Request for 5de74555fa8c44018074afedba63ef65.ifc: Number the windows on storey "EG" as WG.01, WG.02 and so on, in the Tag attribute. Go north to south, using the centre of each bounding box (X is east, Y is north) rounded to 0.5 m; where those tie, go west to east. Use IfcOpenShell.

First a look at what the model holds.

```python
import ifcopenshell
import ifcopenshell.util.element
import ifcopenshell.util.placement

model = ifcopenshell.open("5de74555fa8c44018074afedba63ef65.ifc")
print(model.schema)
storey = next(s for s in model.by_type("IfcBuildingStorey") if s.Name == "EG")
windows = [e for e in ifcopenshell.util.element.get_decomposition(storey) if e.is_a("IfcWindow")]
for e in sorted(windows, key=lambda e: e.id()):
    origin = ifcopenshell.util.placement.get_local_placement(e.ObjectPlacement)[:3, 3]
    print(e.id(), e.Tag, e.Name, origin.round(2) + 0.0, sep=" | ")
```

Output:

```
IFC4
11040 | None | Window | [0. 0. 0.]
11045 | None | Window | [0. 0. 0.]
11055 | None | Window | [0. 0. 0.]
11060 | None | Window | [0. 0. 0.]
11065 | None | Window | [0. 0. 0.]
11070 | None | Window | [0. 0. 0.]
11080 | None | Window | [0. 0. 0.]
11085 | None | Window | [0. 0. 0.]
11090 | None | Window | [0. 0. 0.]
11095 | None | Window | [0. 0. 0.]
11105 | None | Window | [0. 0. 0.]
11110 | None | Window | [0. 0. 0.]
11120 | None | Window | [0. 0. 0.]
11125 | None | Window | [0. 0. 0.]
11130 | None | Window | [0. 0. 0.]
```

```python
import ifcopenshell
import ifcopenshell.geom
import ifcopenshell.util.element
import ifcopenshell.util.shape

model = ifcopenshell.open("5de74555fa8c44018074afedba63ef65.ifc")
settings = ifcopenshell.geom.settings()
settings.set("use-world-coords", True)


def centre(element):
    shape = ifcopenshell.geom.create_shape(settings, element)
    return ifcopenshell.util.shape.get_bbox_centroid(shape.geometry)


storey = next(s for s in model.by_type("IfcBuildingStorey") if s.Name == "EG")
windows = [e for e in ifcopenshell.util.element.get_decomposition(storey) if e.is_a("IfcWindow")]

# Insertion points can sit at a corner or the storey origin, so sort by the geometry (in metres).
centres = {e: centre(e) for e in windows}
windows.sort(key=lambda e: (-round(centres[e][1] / 0.5), centres[e][0]))

for i, e in enumerate(windows, start=1):
    number = f"WG.{i:02d}"
    e.Tag = number
    print(e.id(), number)

model.write("5de74555fa8c44018074afedba63ef65_updated.ifc")
```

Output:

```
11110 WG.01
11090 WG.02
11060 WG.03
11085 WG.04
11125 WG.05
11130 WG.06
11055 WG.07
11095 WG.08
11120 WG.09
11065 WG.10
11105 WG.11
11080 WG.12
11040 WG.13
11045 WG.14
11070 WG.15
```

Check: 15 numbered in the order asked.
